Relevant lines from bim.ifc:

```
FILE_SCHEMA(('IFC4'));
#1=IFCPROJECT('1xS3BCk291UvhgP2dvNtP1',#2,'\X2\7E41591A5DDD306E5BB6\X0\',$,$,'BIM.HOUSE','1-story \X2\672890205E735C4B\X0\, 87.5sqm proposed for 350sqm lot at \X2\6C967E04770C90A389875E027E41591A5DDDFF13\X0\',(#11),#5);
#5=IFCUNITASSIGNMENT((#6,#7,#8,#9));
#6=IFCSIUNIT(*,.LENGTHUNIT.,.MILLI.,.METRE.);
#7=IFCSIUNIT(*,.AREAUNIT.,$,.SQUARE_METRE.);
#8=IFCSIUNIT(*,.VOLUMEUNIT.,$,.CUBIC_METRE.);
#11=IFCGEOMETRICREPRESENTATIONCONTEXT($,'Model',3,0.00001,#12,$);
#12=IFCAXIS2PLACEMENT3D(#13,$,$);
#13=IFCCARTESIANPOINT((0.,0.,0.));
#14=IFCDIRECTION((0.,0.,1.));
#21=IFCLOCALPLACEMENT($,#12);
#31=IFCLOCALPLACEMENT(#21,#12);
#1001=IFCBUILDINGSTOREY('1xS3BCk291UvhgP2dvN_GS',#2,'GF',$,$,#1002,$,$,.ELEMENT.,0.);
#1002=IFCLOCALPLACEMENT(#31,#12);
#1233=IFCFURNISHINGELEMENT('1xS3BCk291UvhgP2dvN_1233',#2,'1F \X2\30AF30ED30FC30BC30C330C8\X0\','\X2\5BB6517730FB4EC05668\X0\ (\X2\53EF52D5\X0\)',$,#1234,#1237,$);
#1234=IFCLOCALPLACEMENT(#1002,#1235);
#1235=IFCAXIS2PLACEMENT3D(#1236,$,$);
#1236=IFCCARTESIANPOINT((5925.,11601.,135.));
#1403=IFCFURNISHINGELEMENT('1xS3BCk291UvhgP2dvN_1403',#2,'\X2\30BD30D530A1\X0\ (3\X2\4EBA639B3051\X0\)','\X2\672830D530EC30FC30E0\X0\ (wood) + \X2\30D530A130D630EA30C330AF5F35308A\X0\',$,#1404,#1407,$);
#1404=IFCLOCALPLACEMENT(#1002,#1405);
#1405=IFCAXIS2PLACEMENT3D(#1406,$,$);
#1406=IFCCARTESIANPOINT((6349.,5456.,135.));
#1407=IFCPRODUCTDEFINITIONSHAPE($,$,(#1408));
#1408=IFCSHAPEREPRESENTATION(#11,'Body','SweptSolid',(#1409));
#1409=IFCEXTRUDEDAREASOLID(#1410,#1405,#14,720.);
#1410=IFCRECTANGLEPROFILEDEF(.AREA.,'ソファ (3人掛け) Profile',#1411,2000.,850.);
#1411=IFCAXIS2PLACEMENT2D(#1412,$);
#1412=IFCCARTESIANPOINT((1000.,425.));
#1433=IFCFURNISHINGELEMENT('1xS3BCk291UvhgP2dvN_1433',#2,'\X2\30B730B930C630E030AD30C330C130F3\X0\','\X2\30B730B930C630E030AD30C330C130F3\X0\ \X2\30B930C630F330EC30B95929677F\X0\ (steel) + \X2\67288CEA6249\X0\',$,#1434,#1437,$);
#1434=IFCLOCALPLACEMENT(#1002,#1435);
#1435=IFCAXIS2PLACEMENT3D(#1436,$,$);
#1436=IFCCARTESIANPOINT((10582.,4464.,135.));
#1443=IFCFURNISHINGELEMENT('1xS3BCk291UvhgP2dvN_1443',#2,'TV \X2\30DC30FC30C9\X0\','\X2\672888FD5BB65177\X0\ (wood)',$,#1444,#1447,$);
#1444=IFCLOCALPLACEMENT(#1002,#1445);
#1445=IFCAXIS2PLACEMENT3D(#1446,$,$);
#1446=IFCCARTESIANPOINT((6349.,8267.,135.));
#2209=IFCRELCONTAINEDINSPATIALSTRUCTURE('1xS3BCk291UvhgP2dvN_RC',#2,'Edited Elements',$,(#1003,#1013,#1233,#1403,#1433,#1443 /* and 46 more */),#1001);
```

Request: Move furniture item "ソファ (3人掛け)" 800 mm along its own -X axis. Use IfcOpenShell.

```python
import ifcopenshell
import ifcopenshell.api.geometry
import ifcopenshell.util.placement
import ifcopenshell.util.unit

model = ifcopenshell.open("bim.ifc")
unit_scale = ifcopenshell.util.unit.calculate_unit_scale(model)

item = model.by_id(1403)
matrix = ifcopenshell.util.placement.get_local_placement(item.ObjectPlacement)
matrix[:3, 3] -= matrix[:3, 0] * 0.8 / unit_scale
ifcopenshell.api.geometry.edit_object_placement(model, product=item, matrix=matrix, is_si=False)

print(ifcopenshell.util.placement.get_local_placement(item.ObjectPlacement).round(3) + 0.0)

model.write("bim_updated.ifc")
```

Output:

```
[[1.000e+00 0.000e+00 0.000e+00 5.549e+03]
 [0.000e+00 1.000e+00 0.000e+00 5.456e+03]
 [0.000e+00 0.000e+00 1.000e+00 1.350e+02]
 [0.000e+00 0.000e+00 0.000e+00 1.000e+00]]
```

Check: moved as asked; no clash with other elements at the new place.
